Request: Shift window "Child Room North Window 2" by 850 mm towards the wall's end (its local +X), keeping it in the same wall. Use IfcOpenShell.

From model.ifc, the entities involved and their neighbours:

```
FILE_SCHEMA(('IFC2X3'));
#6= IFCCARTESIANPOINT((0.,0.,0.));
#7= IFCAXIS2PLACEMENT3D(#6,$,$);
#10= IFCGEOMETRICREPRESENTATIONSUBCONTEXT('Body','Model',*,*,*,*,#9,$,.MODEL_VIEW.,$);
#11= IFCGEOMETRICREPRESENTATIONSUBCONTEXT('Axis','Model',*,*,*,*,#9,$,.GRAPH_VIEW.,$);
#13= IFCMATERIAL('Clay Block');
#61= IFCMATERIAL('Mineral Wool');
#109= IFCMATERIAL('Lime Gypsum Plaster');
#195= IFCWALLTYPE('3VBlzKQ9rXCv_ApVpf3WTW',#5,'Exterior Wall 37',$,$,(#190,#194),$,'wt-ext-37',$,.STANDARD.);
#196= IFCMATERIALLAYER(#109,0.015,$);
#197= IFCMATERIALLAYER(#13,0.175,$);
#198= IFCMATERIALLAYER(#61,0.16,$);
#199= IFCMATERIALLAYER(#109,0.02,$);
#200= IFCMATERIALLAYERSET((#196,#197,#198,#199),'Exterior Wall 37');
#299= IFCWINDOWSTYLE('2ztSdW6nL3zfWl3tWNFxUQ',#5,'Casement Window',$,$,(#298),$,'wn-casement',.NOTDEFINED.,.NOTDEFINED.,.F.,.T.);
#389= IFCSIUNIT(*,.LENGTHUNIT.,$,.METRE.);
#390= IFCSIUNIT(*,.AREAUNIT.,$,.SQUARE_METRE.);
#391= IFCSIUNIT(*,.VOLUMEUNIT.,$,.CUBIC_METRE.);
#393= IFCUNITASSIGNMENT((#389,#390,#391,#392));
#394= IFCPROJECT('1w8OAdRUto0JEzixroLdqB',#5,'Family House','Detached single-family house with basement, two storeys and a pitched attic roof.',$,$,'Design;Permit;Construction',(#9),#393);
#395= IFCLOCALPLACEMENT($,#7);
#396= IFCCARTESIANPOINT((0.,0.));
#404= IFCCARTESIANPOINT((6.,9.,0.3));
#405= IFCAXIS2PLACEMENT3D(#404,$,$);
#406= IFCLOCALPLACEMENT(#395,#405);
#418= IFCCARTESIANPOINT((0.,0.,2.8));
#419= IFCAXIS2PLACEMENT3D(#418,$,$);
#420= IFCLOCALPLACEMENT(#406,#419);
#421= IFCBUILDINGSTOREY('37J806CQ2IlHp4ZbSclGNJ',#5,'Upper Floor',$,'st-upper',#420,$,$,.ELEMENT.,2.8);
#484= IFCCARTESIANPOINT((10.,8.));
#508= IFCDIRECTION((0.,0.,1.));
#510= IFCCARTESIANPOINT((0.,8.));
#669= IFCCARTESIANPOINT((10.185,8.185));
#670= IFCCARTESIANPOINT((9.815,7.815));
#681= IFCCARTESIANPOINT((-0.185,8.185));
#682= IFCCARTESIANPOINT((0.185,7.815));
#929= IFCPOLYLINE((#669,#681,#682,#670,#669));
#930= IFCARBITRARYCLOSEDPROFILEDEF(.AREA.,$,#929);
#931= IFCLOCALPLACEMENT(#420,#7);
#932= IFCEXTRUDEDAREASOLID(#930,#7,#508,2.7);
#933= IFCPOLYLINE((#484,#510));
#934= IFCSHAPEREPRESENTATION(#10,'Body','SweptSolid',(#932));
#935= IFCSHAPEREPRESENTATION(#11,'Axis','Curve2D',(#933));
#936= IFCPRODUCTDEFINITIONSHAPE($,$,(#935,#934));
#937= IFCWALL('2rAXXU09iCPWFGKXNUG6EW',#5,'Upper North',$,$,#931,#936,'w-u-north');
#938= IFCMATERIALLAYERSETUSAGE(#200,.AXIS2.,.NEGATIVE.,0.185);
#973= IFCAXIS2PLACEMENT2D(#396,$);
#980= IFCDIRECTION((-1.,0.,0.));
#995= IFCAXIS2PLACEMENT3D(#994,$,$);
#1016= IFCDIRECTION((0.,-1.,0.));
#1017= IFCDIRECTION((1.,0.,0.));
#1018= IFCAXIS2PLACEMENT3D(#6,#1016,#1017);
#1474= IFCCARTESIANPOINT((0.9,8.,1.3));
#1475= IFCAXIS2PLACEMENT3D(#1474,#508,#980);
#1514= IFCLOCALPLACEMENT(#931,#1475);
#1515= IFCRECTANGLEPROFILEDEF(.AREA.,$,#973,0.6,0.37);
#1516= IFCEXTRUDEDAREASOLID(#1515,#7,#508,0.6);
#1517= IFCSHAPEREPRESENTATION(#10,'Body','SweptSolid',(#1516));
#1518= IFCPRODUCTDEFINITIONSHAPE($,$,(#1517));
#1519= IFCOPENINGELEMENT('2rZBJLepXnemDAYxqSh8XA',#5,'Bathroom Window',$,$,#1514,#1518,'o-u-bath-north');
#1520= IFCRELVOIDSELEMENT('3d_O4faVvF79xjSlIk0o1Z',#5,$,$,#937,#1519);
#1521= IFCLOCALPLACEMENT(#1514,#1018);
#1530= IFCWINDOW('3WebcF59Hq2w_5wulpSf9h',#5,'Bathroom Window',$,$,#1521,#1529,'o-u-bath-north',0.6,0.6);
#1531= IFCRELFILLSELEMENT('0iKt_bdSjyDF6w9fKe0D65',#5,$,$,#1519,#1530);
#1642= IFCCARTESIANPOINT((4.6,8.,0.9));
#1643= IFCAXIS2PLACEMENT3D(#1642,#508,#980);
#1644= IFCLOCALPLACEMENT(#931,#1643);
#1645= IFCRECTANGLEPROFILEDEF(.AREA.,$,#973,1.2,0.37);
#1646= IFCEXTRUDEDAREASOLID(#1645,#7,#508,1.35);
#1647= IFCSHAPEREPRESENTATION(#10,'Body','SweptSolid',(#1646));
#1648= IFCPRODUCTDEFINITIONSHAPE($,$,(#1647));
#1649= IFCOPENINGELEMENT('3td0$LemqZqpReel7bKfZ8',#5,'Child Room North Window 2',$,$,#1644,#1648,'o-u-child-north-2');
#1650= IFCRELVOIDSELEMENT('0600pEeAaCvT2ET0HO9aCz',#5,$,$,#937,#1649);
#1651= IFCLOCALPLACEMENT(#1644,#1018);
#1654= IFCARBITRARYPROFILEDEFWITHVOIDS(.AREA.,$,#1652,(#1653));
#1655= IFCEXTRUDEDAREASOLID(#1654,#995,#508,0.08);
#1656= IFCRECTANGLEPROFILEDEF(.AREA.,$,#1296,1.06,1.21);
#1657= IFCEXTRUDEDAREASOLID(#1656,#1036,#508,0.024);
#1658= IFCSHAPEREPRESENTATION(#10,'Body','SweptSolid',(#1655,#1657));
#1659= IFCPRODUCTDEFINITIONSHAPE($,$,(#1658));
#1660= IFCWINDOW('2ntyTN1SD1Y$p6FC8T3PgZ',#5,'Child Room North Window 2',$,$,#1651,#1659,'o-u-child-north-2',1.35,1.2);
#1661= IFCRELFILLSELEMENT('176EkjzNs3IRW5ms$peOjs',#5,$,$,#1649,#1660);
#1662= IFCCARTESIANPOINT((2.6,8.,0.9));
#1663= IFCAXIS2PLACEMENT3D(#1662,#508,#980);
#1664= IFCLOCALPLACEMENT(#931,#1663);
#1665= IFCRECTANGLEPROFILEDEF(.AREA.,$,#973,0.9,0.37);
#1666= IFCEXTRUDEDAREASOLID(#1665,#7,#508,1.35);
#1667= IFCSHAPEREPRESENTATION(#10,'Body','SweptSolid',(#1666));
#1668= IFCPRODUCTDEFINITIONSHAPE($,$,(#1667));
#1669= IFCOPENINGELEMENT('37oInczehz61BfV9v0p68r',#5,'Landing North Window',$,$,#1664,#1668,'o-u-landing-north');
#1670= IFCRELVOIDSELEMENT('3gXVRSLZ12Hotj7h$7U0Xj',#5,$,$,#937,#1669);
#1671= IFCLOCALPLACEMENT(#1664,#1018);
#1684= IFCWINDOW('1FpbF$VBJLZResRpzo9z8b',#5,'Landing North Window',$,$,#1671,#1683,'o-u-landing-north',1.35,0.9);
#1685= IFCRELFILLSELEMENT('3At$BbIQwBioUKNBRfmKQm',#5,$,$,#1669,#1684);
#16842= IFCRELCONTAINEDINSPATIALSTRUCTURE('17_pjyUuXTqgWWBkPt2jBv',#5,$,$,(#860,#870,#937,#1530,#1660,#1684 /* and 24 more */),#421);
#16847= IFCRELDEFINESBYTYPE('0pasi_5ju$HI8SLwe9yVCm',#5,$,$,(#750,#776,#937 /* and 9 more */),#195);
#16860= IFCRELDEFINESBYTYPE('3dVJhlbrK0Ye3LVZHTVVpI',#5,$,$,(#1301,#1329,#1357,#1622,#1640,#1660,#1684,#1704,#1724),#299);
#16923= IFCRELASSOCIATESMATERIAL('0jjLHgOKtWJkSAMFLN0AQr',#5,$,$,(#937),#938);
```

```python
import ifcopenshell
import ifcopenshell.api.geometry
import ifcopenshell.util.placement
import ifcopenshell.util.unit

model = ifcopenshell.open("model.ifc")
unit_scale = ifcopenshell.util.unit.calculate_unit_scale(model)

window = model.by_guid("2ntyTN1SD1Y$p6FC8T3PgZ")
opening = window.FillsVoids[0].RelatingOpeningElement
wall = opening.VoidsElements[0].RelatingBuildingElement

wall_matrix = ifcopenshell.util.placement.get_local_placement(wall.ObjectPlacement)
shift = wall_matrix[:3, 0] * 0.85 / unit_scale
before = ifcopenshell.util.placement.get_local_placement(window.ObjectPlacement)[:3, 3].copy()

# The window is placed relative to its opening, so it follows when the opening moves.
matrix = ifcopenshell.util.placement.get_local_placement(opening.ObjectPlacement)
matrix[:3, 3] += shift
ifcopenshell.api.geometry.edit_object_placement(
    model, product=opening, matrix=matrix, is_si=False, should_transform_children=True
)

after = ifcopenshell.util.placement.get_local_placement(window.ObjectPlacement)[:3, 3]
print("window moved by", (after - before).round(3) + 0.0)

model.write("model_edited.ifc")
```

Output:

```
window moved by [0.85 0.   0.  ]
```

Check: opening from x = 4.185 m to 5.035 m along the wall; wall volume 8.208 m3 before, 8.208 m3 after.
